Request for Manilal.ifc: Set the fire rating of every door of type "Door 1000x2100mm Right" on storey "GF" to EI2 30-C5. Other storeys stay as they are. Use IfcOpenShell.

First a look at what the model holds.

```python
import ifcopenshell
import ifcopenshell.util.element

model = ifcopenshell.open("Manilal.ifc")
print(model.schema)
storey = next(s for s in model.by_type("IfcBuildingStorey") if s.Name == "GF")
doors = [e for e in ifcopenshell.util.element.get_decomposition(storey) if e.is_a("IfcDoor")]
seen = {}
for e in doors:
    element_type = ifcopenshell.util.element.get_type(e)
    key = (element_type.Name if element_type != e and element_type else None, ifcopenshell.util.element.get_pset(e, "Pset_DoorCommon", "FireRating"))
    seen[key] = seen.get(key, 0) + 1
for (name, value), count in sorted(seen.items(), key=str):
    print(count, "x", name, "|", value)
```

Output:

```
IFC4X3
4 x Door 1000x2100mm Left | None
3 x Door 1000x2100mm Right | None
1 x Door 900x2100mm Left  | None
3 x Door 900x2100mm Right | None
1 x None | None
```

```python
import ifcopenshell
import ifcopenshell.api.pset
import ifcopenshell.util.element

model = ifcopenshell.open("Manilal.ifc")

storey = next(s for s in model.by_type("IfcBuildingStorey") if s.Name == "GF")
doors = [e for e in ifcopenshell.util.element.get_decomposition(storey) if e.is_a("IfcDoor")]

count = 0
for e in doors:
    element_type = ifcopenshell.util.element.get_type(e)
    if element_type in (None, e) or element_type.Name != "Door 1000x2100mm Right":
        continue
    # add_pset returns the element's existing set when there is one.
    pset = ifcopenshell.api.pset.add_pset(model, product=e, name="Pset_DoorCommon")
    ifcopenshell.api.pset.edit_pset(model, pset=pset, properties={"FireRating": "EI2 30-C5"})
    count += 1

print(count, "doors updated")

model.write("Manilal_rev.ifc")
```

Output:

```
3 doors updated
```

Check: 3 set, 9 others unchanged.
